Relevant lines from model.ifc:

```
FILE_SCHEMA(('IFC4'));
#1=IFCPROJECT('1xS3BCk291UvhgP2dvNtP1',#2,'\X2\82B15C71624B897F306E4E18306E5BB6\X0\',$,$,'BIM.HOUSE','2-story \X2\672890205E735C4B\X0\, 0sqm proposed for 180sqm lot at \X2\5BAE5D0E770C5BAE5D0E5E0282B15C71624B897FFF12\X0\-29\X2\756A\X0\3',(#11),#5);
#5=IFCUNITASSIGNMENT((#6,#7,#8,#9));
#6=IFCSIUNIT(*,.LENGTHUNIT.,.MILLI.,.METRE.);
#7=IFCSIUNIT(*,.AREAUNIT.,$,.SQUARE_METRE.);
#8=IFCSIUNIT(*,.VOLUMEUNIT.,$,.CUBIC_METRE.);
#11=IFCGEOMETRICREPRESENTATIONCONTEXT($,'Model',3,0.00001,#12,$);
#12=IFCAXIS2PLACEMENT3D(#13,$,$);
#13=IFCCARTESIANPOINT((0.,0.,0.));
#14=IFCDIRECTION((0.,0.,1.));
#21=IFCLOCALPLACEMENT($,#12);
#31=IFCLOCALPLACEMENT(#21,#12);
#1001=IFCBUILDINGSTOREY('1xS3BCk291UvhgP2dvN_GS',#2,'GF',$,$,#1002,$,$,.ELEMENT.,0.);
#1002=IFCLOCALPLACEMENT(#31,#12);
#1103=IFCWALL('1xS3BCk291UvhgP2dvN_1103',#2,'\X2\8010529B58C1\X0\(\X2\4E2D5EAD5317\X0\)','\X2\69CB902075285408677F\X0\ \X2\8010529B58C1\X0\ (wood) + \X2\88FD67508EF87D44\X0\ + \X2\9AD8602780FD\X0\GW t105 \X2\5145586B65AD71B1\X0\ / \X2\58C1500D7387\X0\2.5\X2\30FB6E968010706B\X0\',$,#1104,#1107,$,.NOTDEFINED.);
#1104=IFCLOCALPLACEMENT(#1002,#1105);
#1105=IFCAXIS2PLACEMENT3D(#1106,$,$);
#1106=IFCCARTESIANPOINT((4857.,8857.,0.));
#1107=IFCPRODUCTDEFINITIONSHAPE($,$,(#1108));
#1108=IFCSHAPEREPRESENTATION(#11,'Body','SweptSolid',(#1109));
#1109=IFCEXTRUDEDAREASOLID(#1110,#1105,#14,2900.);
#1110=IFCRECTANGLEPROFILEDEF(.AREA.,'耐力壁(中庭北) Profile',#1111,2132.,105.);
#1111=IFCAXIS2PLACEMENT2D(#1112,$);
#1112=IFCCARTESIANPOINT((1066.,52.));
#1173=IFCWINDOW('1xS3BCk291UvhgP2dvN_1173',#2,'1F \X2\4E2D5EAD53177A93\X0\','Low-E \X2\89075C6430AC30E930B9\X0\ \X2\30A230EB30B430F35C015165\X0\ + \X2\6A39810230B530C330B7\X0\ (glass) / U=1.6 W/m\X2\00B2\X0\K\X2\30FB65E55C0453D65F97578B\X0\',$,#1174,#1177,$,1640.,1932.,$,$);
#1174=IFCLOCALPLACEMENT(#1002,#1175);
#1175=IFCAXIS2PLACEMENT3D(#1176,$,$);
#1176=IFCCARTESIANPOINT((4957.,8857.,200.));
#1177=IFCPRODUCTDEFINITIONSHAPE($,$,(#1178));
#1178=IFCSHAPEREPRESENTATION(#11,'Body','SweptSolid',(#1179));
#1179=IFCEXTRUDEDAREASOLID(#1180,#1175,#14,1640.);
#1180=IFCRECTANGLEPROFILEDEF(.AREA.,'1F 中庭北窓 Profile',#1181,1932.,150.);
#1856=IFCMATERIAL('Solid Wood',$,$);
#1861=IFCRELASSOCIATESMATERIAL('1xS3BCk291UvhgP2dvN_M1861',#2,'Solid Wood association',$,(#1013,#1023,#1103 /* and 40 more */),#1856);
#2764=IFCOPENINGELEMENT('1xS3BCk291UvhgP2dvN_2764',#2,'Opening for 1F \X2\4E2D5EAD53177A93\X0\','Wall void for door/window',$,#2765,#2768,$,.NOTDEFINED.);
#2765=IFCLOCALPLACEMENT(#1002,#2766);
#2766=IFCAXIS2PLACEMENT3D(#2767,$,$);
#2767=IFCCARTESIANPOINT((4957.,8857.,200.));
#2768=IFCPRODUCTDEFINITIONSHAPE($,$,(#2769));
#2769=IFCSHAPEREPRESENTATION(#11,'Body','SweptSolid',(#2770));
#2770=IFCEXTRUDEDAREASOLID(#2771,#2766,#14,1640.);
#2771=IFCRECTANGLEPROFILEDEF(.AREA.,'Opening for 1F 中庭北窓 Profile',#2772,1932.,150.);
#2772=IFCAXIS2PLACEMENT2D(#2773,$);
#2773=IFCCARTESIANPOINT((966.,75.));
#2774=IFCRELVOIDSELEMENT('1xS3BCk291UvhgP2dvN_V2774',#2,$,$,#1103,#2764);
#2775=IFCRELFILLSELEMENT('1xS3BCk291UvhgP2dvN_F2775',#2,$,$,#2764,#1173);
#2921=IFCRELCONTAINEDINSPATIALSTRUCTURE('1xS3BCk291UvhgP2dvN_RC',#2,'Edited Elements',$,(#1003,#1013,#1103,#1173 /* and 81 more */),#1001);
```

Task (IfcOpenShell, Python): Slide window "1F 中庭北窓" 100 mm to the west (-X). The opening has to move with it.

```python
import ifcopenshell
import ifcopenshell.api.geometry
import ifcopenshell.util.placement
import ifcopenshell.util.unit

model = ifcopenshell.open("model.ifc")
unit_scale = ifcopenshell.util.unit.calculate_unit_scale(model)

window = model.by_guid("1xS3BCk291UvhgP2dvN_1173")
opening = window.FillsVoids[0].RelatingOpeningElement
wall = opening.VoidsElements[0].RelatingBuildingElement

wall_matrix = ifcopenshell.util.placement.get_local_placement(wall.ObjectPlacement)
shift = wall_matrix[:3, 0] * -0.1 / unit_scale
before = ifcopenshell.util.placement.get_local_placement(window.ObjectPlacement)[:3, 3].copy()

# The window is not placed relative to its opening, so move both.
for product in (opening, window):
    matrix = ifcopenshell.util.placement.get_local_placement(product.ObjectPlacement)
    matrix[:3, 3] += shift
    ifcopenshell.api.geometry.edit_object_placement(model, product=product, matrix=matrix, is_si=False)

after = ifcopenshell.util.placement.get_local_placement(window.ObjectPlacement)[:3, 3]
print("window moved by", (after - before).round(3) + 0.0)

model.write("model_v2.ifc")
```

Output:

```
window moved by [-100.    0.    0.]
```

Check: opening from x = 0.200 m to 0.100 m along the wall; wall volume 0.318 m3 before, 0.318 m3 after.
